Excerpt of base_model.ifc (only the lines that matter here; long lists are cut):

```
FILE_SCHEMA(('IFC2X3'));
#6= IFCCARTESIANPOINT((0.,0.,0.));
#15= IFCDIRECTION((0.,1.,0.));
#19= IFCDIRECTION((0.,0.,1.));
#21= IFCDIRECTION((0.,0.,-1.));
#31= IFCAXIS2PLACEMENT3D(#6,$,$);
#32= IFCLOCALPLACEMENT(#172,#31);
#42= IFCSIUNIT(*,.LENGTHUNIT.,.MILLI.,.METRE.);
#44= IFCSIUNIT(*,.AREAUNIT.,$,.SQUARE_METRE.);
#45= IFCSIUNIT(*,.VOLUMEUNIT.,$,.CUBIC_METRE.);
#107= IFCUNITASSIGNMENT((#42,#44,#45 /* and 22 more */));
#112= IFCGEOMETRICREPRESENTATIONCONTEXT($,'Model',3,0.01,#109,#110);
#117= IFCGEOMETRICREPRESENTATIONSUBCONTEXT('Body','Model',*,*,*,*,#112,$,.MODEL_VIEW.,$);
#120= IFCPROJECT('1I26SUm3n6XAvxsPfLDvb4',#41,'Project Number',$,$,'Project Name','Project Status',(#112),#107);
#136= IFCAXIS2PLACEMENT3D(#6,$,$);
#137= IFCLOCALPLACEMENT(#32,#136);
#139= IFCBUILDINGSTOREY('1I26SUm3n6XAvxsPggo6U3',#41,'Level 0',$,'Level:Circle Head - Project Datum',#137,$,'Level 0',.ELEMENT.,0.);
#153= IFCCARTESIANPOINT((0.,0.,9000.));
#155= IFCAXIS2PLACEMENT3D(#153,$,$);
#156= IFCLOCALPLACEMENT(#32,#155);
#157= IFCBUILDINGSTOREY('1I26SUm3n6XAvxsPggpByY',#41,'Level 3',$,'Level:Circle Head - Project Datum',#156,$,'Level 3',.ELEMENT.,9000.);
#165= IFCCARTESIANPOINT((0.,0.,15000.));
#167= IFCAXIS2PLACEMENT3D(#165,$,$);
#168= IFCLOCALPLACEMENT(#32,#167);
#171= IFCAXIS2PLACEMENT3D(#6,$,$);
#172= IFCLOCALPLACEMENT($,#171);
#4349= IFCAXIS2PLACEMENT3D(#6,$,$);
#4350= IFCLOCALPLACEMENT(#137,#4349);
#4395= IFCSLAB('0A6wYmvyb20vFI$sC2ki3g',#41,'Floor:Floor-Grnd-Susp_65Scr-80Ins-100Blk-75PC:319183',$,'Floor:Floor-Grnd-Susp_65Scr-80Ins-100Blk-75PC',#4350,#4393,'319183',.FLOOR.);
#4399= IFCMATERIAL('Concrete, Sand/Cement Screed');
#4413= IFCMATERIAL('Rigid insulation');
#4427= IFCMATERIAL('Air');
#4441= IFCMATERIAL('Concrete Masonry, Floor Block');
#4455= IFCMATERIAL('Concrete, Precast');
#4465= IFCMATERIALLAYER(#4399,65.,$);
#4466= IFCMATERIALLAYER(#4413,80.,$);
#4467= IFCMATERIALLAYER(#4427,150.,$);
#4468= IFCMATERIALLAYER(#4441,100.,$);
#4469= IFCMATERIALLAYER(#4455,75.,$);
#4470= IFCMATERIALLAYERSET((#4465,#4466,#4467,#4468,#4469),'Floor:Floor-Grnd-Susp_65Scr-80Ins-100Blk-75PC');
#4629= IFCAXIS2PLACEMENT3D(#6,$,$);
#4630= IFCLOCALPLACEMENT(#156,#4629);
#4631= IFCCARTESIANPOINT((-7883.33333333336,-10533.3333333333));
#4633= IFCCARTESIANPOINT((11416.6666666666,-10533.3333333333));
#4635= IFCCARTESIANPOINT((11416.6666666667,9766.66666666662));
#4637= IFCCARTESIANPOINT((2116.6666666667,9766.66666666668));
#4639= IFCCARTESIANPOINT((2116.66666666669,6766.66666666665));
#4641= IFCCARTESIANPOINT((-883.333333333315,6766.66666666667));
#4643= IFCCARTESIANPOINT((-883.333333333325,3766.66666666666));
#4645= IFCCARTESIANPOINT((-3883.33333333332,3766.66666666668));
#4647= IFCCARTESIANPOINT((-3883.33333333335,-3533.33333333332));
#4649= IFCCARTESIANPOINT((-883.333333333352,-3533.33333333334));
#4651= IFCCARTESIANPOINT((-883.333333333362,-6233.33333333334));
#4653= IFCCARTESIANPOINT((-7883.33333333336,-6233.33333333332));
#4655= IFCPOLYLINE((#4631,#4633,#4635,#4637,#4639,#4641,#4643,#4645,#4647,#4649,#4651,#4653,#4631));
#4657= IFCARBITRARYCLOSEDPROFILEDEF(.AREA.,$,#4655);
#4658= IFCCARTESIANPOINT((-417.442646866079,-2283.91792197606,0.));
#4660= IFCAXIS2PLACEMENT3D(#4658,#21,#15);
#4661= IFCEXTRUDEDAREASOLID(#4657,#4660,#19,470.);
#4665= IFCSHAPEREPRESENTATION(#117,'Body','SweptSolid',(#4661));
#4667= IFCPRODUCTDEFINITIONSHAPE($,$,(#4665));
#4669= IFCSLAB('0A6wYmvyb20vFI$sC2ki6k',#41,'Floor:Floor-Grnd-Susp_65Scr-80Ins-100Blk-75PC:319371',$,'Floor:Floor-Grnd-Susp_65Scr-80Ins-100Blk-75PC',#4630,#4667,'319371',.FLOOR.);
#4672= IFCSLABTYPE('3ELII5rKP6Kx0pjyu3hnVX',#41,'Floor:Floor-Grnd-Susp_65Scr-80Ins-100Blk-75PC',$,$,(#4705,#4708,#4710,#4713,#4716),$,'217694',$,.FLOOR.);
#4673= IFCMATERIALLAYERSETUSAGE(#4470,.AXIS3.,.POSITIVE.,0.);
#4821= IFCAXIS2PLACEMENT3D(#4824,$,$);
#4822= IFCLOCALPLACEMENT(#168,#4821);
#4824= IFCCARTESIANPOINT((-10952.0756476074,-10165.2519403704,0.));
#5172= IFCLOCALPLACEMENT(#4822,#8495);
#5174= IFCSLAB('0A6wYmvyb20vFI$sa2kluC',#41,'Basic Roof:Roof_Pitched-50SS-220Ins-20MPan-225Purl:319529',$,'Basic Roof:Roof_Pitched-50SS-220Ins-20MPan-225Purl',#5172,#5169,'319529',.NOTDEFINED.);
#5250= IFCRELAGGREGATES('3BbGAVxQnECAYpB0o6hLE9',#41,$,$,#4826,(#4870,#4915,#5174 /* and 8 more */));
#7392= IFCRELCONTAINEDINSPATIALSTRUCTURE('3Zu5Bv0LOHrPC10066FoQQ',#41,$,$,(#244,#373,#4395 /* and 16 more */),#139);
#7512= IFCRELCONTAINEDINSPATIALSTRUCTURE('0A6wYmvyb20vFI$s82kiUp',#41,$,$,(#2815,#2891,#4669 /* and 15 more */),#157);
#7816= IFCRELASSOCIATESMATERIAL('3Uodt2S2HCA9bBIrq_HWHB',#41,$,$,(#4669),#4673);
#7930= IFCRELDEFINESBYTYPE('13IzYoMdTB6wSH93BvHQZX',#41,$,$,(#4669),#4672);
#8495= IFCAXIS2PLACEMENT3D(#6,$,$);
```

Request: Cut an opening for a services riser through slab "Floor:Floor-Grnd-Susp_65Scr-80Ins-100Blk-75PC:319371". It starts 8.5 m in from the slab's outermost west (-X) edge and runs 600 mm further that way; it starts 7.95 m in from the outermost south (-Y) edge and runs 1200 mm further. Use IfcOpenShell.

```python
import numpy as np
import ifcopenshell
import ifcopenshell.api.feature
import ifcopenshell.api.geometry
import ifcopenshell.api.root
import ifcopenshell.geom
import ifcopenshell.util.placement
import ifcopenshell.util.representation
import ifcopenshell.util.shape
import ifcopenshell.util.unit

model = ifcopenshell.open("base_model.ifc")
unit_scale = ifcopenshell.util.unit.calculate_unit_scale(model)
settings = ifcopenshell.geom.settings()


def volume(element):
    """Net volume in cubic metres, openings subtracted."""
    shape = ifcopenshell.geom.create_shape(settings, element)
    return ifcopenshell.util.shape.get_volume(shape.geometry)


slab = model.by_id(4669)
before = volume(slab)

# Extent in the slab's own axes, in metres. The edges named are its -X and -Y sides.
slab_shape = ifcopenshell.geom.create_shape(settings, slab)
vertices = ifcopenshell.util.shape.get_vertices(slab_shape.geometry)
x_min, y_min, bottom = vertices.min(axis=0)
top = vertices[:, 2].max()

opening = ifcopenshell.api.root.create_entity(model, ifc_class="IfcOpeningElement", name="Services riser opening")
context = ifcopenshell.util.representation.get_context(model, "Model", "Body", "MODEL_VIEW")
width, depth = 0.6, 1.2
outline = [(0.0, 0.0), (width, 0.0), (width, depth), (0.0, depth), (0.0, 0.0)]
# Overshoot both faces by 50 mm so the cut is clean.
shape = ifcopenshell.api.geometry.add_slab_representation(
    model, context=context, depth=top - bottom + 0.1, polyline=outline
)
ifcopenshell.api.geometry.assign_representation(model, product=opening, representation=shape)

matrix = ifcopenshell.util.placement.get_local_placement(slab.ObjectPlacement)
matrix[:, 3] = matrix @ np.append(np.array([x_min + 8.5, y_min + 7.95, bottom - 0.05]) / unit_scale, 1.0)
ifcopenshell.api.geometry.edit_object_placement(model, product=opening, matrix=matrix, is_si=False)
ifcopenshell.api.feature.add_feature(model, feature=opening, element=slab)

after = volume(slab)

print(f"slab volume {before:.3f} -> {after:.3f} m3")

model.write("base_model_rev.ifc")
```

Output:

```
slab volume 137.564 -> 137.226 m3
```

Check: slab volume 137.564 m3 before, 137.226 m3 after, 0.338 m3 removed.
